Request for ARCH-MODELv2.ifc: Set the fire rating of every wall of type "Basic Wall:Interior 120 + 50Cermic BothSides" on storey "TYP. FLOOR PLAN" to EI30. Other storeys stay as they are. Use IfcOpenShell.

First a look at what the model holds.

```python
import ifcopenshell
import ifcopenshell.util.element

model = ifcopenshell.open("ARCH-MODELv2.ifc")
print(model.schema)
storey = next(s for s in model.by_type("IfcBuildingStorey") if s.Name == "TYP. FLOOR PLAN")
walls = [e for e in ifcopenshell.util.element.get_decomposition(storey) if e.is_a("IfcWall")]
seen = {}
for e in walls:
    element_type = ifcopenshell.util.element.get_type(e)
    key = (element_type.Name if element_type != e and element_type else None, ifcopenshell.util.element.get_pset(e, "Pset_WallCommon", "FireRating"))
    seen[key] = seen.get(key, 0) + 1
for (name, value), count in sorted(seen.items(), key=str):
    print(count, "x", name, "|", value)
```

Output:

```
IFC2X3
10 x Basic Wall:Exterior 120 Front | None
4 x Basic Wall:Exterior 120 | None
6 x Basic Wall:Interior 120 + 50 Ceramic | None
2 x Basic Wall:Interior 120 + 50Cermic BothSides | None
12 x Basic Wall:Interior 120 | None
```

```python
import ifcopenshell
import ifcopenshell.api.pset
import ifcopenshell.util.element

model = ifcopenshell.open("ARCH-MODELv2.ifc")

storey = next(s for s in model.by_type("IfcBuildingStorey") if s.Name == "TYP. FLOOR PLAN")
walls = [e for e in ifcopenshell.util.element.get_decomposition(storey) if e.is_a("IfcWall")]

count = 0
for e in walls:
    element_type = ifcopenshell.util.element.get_type(e)
    if element_type in (None, e) or element_type.Name != "Basic Wall:Interior 120 + 50Cermic BothSides":
        continue
    # add_pset returns the element's existing set when there is one.
    pset = ifcopenshell.api.pset.add_pset(model, product=e, name="Pset_WallCommon")
    ifcopenshell.api.pset.edit_pset(model, pset=pset, properties={"FireRating": "EI30"})
    count += 1

print(count, "walls updated")

model.write("ARCH-MODELv2_updated.ifc")
```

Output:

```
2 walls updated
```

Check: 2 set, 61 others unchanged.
